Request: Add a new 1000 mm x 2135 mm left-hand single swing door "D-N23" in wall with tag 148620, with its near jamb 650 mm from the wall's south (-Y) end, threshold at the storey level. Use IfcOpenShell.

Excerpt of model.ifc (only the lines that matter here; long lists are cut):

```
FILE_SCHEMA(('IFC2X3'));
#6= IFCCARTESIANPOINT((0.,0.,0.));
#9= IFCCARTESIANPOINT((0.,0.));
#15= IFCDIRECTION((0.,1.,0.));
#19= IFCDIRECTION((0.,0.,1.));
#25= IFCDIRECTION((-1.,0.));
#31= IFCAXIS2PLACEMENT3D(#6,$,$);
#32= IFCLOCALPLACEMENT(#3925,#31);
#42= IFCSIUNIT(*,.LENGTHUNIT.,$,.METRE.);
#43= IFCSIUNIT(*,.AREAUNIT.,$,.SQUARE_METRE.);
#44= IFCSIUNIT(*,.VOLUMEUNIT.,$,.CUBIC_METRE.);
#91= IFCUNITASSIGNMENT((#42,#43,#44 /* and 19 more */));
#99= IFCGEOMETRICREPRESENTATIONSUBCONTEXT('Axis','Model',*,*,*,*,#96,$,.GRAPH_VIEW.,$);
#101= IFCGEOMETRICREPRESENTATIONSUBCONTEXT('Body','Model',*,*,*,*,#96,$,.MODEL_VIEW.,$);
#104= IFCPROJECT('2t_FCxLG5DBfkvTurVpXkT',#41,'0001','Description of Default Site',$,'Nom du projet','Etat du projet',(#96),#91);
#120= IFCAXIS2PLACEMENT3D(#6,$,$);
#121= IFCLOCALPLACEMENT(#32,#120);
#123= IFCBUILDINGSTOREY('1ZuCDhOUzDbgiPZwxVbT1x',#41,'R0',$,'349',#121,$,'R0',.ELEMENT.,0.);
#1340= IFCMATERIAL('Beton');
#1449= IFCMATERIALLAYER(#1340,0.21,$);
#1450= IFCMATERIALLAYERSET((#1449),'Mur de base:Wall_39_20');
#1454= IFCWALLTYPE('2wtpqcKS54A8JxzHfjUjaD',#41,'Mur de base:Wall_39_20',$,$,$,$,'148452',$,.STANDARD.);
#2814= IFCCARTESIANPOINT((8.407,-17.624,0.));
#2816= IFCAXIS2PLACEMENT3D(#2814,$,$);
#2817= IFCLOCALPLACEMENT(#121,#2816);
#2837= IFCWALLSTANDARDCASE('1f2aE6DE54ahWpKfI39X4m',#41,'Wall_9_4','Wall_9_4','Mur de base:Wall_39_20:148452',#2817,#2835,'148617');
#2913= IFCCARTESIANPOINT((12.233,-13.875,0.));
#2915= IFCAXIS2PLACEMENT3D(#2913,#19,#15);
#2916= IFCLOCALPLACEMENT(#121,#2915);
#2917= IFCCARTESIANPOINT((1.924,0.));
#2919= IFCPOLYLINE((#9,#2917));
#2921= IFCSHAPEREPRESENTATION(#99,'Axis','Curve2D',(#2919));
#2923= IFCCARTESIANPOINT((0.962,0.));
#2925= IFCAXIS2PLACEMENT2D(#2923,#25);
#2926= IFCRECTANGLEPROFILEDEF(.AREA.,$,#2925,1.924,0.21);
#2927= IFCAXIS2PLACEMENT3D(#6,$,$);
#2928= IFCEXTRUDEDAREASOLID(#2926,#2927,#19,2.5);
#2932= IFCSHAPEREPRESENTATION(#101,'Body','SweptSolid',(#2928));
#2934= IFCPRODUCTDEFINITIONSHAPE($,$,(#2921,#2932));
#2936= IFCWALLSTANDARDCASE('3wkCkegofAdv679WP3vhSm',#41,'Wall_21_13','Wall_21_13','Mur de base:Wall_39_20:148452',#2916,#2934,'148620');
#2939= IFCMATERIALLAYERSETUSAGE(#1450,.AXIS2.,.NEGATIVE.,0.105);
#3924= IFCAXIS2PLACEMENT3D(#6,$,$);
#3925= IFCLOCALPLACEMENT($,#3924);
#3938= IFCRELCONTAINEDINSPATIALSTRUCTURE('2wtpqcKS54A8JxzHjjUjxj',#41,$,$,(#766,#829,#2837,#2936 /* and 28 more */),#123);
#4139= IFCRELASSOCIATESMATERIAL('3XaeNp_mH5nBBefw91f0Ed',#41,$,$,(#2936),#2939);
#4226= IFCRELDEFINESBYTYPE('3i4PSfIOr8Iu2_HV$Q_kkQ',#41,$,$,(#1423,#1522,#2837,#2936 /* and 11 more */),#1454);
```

```python
import numpy as np
import ifcopenshell
import ifcopenshell.api.feature
import ifcopenshell.api.geometry
import ifcopenshell.api.root
import ifcopenshell.api.spatial
import ifcopenshell.api.type
import ifcopenshell.geom
import ifcopenshell.util.element
import ifcopenshell.util.placement
import ifcopenshell.util.representation
import ifcopenshell.util.shape
import ifcopenshell.util.unit

model = ifcopenshell.open("model.ifc")
unit_scale = ifcopenshell.util.unit.calculate_unit_scale(model)
settings = ifcopenshell.geom.settings()


def volume(element):
    """Net volume in cubic metres, openings subtracted."""
    shape = ifcopenshell.geom.create_shape(settings, element)
    return ifcopenshell.util.shape.get_volume(shape.geometry)


wall = model.by_guid("3wkCkegofAdv679WP3vhSm")
storey = ifcopenshell.util.element.get_container(wall, ifc_class="IfcBuildingStorey")
context = ifcopenshell.util.representation.get_context(model, "Model", "Body", "MODEL_VIEW")
before = volume(wall)

width, height, from_end, sill = 1, 2.135, 0.65, 0.0  # metres

# The wall runs along its own X axis, and the end named is its -X end.
wall_shape = ifcopenshell.geom.create_shape(settings, wall)
x, y, z = ifcopenshell.util.shape.get_vertices(wall_shape.geometry).T
start = x.min() + from_end
face, thickness = float(y.min()), float(y.max() - y.min())
wall_matrix = ifcopenshell.util.placement.get_local_placement(wall.ObjectPlacement)
level = ifcopenshell.util.placement.get_local_placement(storey.ObjectPlacement)[2, 3]


def in_wall(x, y):
    """Placement at x, y metres in the wall's axes, at sill height."""
    matrix = wall_matrix.copy()
    matrix[:, 3] = wall_matrix @ np.array([x / unit_scale, y / unit_scale, 0.0, 1.0])
    matrix[2, 3] = level + sill / unit_scale
    return matrix


# Opening: a box that overshoots both wall faces by 50 mm.
opening = ifcopenshell.api.root.create_entity(model, ifc_class="IfcOpeningElement")
box = ifcopenshell.api.geometry.add_wall_representation(
    model, context=context, length=width, height=height, thickness=thickness + 0.1
)
ifcopenshell.api.geometry.assign_representation(model, product=opening, representation=box)
ifcopenshell.api.geometry.edit_object_placement(model, product=opening, matrix=in_wall(start, face - 0.05), is_si=False)
ifcopenshell.api.feature.add_feature(model, feature=opening, element=wall)

door = ifcopenshell.api.root.create_entity(model, ifc_class="IfcDoor", name="D-N23")
door.OverallWidth, door.OverallHeight = width / unit_scale, height / unit_scale
body = ifcopenshell.api.geometry.add_door_representation(
    model,
    context=context,
    overall_width=door.OverallWidth,
    overall_height=door.OverallHeight,
    operation_type="SINGLE_SWING_LEFT",
    lining_properties={"LiningDepth": thickness / unit_scale, "ThresholdDepth": thickness / unit_scale},
)
ifcopenshell.api.geometry.assign_representation(model, product=door, representation=body)
ifcopenshell.api.spatial.assign_container(model, products=[door], relating_structure=storey)
fills = ifcopenshell.api.feature.add_filling(model, opening=opening, element=door)
fills.OwnerHistory = door.OwnerHistory  # required in IFC2X3

# IFC2X3 keeps the operation on the door style.
style = ifcopenshell.api.root.create_entity(model, ifc_class="IfcDoorStyle", name="D-N23")
style.OperationType, style.ConstructionType = "SINGLE_SWING_LEFT", "NOTDEFINED"
style.ParameterTakesPrecedence = style.Sizeable = False
ifcopenshell.api.type.assign_type(model, related_objects=[door], relating_type=style)

# The lining spans the wall, so the door starts at the wall face.
ifcopenshell.api.geometry.edit_object_placement(model, product=door, matrix=in_wall(start, face), is_si=False)

after = volume(wall)

print(f"wall volume {before:.3f} -> {after:.3f} m3")

model.write("model_rev.ifc")
```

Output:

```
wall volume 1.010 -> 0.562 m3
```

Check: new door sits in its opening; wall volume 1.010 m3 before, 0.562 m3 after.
